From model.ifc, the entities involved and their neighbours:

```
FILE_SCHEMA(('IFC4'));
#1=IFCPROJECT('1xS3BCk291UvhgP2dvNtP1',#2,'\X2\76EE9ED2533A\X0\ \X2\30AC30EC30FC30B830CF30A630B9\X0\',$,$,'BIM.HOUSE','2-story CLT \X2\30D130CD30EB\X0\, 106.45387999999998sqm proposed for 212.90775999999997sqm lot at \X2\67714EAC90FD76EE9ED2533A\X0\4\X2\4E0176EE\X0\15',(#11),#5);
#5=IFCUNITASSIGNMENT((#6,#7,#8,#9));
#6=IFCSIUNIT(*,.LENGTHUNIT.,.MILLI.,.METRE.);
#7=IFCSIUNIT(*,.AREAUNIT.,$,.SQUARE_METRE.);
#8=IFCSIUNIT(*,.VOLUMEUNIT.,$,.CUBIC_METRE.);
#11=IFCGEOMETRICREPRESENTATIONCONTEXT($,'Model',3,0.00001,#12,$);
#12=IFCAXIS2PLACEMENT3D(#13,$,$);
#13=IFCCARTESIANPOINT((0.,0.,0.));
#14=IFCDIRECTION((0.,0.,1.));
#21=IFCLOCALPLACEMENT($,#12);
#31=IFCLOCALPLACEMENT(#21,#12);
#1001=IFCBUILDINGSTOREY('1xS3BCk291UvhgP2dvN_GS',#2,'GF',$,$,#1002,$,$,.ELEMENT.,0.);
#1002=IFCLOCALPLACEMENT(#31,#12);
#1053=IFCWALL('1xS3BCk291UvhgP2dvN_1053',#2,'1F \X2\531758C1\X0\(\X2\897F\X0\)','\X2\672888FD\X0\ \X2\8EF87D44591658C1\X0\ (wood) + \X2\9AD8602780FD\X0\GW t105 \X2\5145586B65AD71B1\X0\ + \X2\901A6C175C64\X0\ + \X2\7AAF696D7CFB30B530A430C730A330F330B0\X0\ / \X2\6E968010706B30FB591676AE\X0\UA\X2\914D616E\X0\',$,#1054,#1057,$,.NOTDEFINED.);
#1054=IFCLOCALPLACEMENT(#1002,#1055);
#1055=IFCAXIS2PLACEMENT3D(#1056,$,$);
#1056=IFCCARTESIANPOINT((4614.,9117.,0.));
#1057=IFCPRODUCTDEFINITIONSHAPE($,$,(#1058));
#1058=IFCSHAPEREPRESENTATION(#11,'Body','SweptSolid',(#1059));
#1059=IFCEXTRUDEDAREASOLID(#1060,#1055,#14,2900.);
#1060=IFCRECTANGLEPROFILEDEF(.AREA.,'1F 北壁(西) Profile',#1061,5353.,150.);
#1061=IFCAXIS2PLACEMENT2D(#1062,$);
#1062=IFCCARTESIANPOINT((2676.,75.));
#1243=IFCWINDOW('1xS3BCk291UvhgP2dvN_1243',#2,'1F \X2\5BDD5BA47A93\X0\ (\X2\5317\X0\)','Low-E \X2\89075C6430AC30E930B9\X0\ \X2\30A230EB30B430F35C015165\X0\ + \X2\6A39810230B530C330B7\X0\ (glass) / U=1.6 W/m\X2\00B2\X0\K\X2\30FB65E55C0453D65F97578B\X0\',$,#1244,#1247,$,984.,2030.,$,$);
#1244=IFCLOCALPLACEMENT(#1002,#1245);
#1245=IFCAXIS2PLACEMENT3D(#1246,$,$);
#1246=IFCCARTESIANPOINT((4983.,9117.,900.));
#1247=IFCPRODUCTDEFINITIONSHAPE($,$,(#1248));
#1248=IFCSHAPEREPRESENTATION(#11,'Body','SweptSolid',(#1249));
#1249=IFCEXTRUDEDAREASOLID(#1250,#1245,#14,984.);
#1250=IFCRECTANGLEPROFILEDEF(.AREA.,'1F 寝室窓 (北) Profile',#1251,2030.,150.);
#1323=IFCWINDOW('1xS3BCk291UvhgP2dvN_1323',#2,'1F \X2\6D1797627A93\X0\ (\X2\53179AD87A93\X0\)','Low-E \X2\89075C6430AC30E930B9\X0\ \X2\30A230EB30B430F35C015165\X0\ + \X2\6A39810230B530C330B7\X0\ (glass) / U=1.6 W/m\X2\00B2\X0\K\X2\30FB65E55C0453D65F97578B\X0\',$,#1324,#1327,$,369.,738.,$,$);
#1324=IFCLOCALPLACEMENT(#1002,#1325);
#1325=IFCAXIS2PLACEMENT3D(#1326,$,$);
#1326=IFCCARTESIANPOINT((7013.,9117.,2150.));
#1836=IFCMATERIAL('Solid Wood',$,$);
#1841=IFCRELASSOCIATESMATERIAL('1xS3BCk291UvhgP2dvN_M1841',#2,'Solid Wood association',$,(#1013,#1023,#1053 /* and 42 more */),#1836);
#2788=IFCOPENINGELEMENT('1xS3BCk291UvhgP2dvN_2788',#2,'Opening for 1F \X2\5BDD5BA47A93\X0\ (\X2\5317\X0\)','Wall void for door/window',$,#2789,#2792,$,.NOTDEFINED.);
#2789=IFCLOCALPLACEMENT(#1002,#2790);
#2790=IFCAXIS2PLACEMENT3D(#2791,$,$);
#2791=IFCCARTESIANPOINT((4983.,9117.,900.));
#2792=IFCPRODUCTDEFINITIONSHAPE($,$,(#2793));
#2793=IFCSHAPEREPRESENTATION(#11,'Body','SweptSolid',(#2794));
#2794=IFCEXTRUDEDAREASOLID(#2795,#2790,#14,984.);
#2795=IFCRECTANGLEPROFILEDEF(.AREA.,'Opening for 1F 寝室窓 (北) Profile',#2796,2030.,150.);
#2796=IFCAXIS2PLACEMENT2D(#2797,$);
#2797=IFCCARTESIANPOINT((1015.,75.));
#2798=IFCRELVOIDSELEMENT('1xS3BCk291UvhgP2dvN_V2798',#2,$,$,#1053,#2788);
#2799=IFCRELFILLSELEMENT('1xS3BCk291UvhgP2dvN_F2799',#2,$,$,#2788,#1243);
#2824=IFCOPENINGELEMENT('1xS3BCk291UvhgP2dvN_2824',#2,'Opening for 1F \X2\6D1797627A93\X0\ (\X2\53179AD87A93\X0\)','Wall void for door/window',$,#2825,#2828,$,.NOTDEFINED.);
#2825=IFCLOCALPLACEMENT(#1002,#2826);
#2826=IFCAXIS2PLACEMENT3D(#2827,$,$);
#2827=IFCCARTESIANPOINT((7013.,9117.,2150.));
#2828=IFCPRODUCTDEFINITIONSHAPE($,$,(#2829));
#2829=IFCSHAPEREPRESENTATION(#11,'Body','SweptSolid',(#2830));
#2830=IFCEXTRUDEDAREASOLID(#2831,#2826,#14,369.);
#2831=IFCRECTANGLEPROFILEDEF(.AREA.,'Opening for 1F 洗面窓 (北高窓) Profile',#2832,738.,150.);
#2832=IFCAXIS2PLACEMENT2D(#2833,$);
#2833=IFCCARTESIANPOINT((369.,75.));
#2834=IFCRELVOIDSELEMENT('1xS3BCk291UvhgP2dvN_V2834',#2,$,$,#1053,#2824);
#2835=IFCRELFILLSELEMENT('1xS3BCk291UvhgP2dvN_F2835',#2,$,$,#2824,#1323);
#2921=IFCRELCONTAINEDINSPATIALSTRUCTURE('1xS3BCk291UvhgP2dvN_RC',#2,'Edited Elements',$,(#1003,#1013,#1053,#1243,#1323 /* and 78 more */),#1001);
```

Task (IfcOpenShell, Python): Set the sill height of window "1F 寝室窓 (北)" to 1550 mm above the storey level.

```python
import numpy as np
import ifcopenshell
import ifcopenshell.api.geometry
import ifcopenshell.geom
import ifcopenshell.util.element
import ifcopenshell.util.placement
import ifcopenshell.util.shape
import ifcopenshell.util.unit

model = ifcopenshell.open("model.ifc")
unit_scale = ifcopenshell.util.unit.calculate_unit_scale(model)

window = model.by_guid("1xS3BCk291UvhgP2dvN_1243")
opening = window.FillsVoids[0].RelatingOpeningElement
storey = ifcopenshell.util.element.get_container(window, ifc_class="IfcBuildingStorey")
level = ifcopenshell.util.placement.get_local_placement(storey.ObjectPlacement)[2, 3]

# The opening's origin need not be at the sill, so measure its lowest point.
shape = ifcopenshell.geom.create_shape(ifcopenshell.geom.settings(), opening)
bottom = ifcopenshell.util.shape.get_shape_bottom_elevation(shape, shape.geometry) / unit_scale
dz = level + 1.55 / unit_scale - bottom

shift = np.array([0.0, 0.0, dz])
# The window is not placed relative to its opening, so move both.
for product in (opening, window):
    matrix = ifcopenshell.util.placement.get_local_placement(product.ObjectPlacement)
    matrix[:3, 3] += shift
    ifcopenshell.api.geometry.edit_object_placement(model, product=product, matrix=matrix, is_si=False)

print(f"moved by {dz * unit_scale:+.3f} m")

model.write("model-out.ifc")
```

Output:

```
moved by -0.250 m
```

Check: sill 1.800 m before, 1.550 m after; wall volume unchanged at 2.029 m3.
